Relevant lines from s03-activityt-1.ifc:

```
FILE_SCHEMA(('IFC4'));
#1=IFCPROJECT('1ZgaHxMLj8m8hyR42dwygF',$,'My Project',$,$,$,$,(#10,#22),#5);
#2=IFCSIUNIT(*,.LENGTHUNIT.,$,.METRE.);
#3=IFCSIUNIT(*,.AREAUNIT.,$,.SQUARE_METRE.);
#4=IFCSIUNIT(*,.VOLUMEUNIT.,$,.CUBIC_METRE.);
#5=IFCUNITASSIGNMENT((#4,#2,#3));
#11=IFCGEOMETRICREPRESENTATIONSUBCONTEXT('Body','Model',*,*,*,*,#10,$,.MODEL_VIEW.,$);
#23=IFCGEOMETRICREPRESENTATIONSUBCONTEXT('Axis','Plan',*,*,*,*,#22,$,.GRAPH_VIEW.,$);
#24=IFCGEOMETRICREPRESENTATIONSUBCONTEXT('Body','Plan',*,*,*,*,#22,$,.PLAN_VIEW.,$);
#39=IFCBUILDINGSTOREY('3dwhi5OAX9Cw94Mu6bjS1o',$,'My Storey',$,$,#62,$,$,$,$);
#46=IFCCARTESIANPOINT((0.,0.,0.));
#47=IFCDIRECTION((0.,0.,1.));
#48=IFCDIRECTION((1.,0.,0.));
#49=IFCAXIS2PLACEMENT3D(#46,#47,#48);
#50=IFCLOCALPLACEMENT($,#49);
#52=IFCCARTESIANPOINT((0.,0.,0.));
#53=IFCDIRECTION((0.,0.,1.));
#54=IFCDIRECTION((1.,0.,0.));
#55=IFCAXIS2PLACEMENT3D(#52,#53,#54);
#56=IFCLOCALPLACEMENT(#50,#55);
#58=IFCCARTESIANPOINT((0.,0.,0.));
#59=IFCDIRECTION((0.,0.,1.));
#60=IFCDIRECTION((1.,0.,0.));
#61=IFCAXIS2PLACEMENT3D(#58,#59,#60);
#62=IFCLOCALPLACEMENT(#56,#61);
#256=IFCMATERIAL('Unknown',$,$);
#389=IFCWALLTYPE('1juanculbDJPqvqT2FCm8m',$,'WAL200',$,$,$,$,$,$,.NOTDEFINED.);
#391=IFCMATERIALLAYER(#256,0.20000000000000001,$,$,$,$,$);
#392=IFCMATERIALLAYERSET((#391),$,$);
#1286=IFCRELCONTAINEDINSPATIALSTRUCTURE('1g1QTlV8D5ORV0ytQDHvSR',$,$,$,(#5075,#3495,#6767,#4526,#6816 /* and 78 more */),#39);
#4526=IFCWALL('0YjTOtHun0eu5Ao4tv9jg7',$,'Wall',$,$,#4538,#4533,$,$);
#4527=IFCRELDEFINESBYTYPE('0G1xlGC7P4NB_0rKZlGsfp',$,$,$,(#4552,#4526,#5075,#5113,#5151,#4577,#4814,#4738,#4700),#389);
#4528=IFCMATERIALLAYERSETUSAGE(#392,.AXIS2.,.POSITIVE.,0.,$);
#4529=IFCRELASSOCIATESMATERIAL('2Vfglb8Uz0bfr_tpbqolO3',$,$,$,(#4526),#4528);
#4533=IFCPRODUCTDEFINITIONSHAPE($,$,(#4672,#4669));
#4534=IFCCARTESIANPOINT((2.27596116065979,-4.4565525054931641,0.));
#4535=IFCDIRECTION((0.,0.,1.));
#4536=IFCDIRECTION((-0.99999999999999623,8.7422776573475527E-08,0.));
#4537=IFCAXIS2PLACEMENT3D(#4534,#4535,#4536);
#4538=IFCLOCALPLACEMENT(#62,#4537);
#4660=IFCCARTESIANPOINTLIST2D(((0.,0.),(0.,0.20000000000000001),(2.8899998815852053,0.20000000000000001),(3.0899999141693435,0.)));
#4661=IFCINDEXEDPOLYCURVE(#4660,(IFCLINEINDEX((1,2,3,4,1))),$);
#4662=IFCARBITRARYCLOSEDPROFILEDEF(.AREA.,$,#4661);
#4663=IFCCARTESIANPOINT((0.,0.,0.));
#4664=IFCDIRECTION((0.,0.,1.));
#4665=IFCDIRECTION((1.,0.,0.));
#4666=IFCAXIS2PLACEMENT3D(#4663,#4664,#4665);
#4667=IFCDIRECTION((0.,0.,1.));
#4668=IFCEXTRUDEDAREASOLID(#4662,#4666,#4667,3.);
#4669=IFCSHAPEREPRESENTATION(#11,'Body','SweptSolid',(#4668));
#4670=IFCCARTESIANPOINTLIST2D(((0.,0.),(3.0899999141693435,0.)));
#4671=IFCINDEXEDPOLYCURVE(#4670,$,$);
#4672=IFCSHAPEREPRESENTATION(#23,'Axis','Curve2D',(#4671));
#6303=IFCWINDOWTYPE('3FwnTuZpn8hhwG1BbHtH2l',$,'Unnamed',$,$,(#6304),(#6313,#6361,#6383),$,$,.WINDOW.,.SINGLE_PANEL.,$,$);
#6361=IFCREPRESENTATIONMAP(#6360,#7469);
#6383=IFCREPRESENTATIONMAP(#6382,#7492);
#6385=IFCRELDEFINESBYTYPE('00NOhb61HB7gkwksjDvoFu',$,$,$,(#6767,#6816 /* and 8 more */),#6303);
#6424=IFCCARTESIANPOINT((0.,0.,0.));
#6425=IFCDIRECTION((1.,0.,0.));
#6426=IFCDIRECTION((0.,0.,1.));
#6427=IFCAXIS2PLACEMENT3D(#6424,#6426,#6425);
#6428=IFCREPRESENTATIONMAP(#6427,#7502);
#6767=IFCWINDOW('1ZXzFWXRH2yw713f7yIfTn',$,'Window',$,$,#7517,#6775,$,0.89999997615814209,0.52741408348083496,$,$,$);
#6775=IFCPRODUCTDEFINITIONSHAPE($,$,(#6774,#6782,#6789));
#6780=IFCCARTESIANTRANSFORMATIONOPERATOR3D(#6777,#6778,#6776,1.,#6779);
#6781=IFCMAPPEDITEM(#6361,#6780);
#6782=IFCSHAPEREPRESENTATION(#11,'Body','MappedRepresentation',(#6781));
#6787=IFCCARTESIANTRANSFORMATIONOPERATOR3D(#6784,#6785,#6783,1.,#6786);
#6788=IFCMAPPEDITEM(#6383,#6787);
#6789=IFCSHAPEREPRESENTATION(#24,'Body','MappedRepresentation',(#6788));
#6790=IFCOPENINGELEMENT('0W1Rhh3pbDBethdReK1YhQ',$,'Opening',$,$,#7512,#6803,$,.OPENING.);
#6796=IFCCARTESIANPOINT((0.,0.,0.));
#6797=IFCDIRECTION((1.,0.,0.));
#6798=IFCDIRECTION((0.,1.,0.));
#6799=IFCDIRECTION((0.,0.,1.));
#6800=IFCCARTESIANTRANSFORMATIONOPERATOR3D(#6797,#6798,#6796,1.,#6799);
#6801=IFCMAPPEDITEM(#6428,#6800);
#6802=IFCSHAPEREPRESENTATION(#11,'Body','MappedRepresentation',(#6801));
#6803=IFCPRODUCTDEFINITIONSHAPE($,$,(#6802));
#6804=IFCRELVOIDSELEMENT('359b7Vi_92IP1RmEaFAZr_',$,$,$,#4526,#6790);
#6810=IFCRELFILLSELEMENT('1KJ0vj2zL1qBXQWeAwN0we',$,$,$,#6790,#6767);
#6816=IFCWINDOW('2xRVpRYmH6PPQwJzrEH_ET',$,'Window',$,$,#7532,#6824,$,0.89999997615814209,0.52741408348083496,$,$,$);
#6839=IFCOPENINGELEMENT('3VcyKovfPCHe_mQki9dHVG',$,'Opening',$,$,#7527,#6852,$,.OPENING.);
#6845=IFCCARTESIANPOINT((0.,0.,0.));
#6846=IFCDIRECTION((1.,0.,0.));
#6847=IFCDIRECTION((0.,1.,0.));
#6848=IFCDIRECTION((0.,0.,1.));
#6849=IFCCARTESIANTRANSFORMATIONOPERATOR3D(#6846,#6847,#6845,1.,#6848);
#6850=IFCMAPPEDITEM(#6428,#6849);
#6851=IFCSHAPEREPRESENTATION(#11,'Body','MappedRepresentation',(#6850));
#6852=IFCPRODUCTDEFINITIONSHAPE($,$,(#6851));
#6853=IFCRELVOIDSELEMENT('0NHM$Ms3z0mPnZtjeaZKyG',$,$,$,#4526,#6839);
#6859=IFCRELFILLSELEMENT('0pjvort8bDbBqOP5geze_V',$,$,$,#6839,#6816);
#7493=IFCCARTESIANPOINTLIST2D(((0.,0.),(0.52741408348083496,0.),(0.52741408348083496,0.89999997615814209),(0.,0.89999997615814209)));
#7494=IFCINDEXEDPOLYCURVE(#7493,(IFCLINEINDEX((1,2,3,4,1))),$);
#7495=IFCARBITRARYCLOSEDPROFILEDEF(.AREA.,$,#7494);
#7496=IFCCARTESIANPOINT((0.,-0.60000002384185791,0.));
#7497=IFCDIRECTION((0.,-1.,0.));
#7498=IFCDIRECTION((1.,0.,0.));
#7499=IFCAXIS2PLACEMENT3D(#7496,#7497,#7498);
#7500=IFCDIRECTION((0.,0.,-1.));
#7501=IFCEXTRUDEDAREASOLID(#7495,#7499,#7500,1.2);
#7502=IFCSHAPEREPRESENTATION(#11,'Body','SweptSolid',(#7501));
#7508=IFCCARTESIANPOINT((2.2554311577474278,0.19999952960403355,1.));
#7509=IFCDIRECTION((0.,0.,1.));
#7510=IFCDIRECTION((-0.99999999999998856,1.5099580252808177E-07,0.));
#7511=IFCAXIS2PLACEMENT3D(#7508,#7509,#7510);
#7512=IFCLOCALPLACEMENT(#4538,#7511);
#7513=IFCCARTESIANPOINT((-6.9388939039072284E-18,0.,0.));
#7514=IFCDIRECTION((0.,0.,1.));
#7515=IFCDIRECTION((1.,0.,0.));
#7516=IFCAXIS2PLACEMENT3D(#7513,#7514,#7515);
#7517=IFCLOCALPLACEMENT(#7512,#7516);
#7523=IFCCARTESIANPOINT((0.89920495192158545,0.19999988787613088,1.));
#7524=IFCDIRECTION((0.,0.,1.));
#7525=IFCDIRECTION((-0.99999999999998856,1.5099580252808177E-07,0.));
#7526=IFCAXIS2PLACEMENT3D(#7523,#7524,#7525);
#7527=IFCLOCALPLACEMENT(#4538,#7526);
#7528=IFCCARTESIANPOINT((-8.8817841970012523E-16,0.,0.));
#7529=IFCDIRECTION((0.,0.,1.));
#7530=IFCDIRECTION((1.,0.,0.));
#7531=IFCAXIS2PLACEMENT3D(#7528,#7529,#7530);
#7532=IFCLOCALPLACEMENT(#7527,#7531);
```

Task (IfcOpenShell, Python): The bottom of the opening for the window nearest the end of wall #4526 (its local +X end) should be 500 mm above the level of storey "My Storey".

```python
import numpy as np
import ifcopenshell
import ifcopenshell.api.geometry
import ifcopenshell.geom
import ifcopenshell.util.element
import ifcopenshell.util.placement
import ifcopenshell.util.shape
import ifcopenshell.util.unit

model = ifcopenshell.open("s03-activityt-1.ifc")
unit_scale = ifcopenshell.util.unit.calculate_unit_scale(model)

window = model.by_guid("1ZXzFWXRH2yw713f7yIfTn")
opening = window.FillsVoids[0].RelatingOpeningElement
storey = ifcopenshell.util.element.get_container(window, ifc_class="IfcBuildingStorey")
level = ifcopenshell.util.placement.get_local_placement(storey.ObjectPlacement)[2, 3]

# The opening's origin need not be at the sill, so measure its lowest point.
shape = ifcopenshell.geom.create_shape(ifcopenshell.geom.settings(), opening)
bottom = ifcopenshell.util.shape.get_shape_bottom_elevation(shape, shape.geometry) / unit_scale
dz = level + 0.5 - bottom

shift = np.array([0.0, 0.0, dz])
# The window is placed relative to its opening, so it follows when the opening moves.
matrix = ifcopenshell.util.placement.get_local_placement(opening.ObjectPlacement)
matrix[:3, 3] += shift
ifcopenshell.api.geometry.edit_object_placement(
    model, product=opening, matrix=matrix, is_si=False, should_transform_children=True
)

print(f"moved by {dz * unit_scale:+.3f} m")

model.write("s03-activityt-1-out.ifc")
```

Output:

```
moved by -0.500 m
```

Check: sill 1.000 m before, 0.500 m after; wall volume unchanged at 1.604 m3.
